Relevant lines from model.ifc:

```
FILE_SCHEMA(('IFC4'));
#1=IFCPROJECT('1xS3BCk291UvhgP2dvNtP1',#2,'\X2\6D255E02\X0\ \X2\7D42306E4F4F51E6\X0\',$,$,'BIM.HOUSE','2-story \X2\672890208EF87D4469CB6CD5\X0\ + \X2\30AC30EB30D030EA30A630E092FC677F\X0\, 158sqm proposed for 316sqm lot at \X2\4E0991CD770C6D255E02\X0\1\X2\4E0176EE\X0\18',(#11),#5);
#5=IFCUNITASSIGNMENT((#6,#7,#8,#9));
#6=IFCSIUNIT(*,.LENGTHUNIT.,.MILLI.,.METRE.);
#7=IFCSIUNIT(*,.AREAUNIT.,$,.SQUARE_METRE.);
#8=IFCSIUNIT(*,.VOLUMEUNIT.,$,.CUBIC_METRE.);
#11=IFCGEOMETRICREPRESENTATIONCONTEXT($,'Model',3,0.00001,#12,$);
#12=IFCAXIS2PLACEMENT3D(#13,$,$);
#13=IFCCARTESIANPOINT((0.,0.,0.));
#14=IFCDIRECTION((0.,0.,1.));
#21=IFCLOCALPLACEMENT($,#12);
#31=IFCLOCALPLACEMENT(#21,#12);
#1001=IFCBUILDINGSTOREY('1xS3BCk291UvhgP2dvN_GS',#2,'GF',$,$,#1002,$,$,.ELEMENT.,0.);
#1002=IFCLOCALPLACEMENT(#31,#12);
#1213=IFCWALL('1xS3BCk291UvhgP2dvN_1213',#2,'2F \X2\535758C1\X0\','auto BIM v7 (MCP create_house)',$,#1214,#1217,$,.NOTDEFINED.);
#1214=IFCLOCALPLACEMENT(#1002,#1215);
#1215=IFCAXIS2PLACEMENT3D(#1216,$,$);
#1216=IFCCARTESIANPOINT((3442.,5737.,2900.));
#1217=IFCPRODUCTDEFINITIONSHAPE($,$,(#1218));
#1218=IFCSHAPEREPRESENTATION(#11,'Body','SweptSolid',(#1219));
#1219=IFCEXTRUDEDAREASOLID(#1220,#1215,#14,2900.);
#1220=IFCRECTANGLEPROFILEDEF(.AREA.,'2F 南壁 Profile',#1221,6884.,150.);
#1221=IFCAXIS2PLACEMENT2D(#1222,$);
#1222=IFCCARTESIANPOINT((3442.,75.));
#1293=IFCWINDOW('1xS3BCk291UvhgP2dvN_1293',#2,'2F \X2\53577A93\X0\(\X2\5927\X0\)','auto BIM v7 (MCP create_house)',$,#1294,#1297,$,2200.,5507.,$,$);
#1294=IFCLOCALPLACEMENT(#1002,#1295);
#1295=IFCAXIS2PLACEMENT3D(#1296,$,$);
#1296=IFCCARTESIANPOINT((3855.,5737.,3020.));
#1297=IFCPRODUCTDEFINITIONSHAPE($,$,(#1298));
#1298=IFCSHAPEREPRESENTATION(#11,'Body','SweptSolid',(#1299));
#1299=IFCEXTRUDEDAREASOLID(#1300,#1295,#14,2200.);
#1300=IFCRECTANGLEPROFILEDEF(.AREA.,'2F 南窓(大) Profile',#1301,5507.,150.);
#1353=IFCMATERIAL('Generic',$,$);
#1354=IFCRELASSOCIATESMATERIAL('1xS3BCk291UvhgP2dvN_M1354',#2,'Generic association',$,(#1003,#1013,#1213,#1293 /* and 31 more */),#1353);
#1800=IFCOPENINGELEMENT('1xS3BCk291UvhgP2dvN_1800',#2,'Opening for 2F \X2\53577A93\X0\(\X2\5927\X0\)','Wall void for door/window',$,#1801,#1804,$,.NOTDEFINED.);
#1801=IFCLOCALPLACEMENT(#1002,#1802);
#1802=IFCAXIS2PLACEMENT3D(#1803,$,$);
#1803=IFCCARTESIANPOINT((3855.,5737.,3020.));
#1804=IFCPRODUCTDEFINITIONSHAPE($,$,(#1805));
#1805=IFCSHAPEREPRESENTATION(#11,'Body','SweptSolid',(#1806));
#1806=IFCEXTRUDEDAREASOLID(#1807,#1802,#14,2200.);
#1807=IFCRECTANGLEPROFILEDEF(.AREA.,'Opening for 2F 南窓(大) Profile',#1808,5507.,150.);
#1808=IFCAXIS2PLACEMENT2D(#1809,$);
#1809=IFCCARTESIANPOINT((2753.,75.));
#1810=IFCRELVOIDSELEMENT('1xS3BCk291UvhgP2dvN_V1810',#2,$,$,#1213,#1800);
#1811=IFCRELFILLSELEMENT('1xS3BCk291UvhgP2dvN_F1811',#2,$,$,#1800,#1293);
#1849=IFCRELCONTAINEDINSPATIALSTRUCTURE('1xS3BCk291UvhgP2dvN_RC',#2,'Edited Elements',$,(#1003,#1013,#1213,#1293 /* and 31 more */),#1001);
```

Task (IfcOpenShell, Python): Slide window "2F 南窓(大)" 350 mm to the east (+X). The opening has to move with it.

```python
import ifcopenshell
import ifcopenshell.api.geometry
import ifcopenshell.util.placement
import ifcopenshell.util.unit

model = ifcopenshell.open("model.ifc")
unit_scale = ifcopenshell.util.unit.calculate_unit_scale(model)

window = model.by_guid("1xS3BCk291UvhgP2dvN_1293")
opening = window.FillsVoids[0].RelatingOpeningElement
wall = opening.VoidsElements[0].RelatingBuildingElement

wall_matrix = ifcopenshell.util.placement.get_local_placement(wall.ObjectPlacement)
shift = wall_matrix[:3, 0] * 0.35 / unit_scale
before = ifcopenshell.util.placement.get_local_placement(window.ObjectPlacement)[:3, 3].copy()

# The window is not placed relative to its opening, so move both.
for product in (opening, window):
    matrix = ifcopenshell.util.placement.get_local_placement(product.ObjectPlacement)
    matrix[:3, 3] += shift
    ifcopenshell.api.geometry.edit_object_placement(model, product=product, matrix=matrix, is_si=False)

after = ifcopenshell.util.placement.get_local_placement(window.ObjectPlacement)[:3, 3]
print("window moved by", (after - before).round(3) + 0.0)

model.write("model-out.ifc")
```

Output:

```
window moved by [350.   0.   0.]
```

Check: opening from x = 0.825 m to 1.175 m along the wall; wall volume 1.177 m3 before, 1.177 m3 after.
